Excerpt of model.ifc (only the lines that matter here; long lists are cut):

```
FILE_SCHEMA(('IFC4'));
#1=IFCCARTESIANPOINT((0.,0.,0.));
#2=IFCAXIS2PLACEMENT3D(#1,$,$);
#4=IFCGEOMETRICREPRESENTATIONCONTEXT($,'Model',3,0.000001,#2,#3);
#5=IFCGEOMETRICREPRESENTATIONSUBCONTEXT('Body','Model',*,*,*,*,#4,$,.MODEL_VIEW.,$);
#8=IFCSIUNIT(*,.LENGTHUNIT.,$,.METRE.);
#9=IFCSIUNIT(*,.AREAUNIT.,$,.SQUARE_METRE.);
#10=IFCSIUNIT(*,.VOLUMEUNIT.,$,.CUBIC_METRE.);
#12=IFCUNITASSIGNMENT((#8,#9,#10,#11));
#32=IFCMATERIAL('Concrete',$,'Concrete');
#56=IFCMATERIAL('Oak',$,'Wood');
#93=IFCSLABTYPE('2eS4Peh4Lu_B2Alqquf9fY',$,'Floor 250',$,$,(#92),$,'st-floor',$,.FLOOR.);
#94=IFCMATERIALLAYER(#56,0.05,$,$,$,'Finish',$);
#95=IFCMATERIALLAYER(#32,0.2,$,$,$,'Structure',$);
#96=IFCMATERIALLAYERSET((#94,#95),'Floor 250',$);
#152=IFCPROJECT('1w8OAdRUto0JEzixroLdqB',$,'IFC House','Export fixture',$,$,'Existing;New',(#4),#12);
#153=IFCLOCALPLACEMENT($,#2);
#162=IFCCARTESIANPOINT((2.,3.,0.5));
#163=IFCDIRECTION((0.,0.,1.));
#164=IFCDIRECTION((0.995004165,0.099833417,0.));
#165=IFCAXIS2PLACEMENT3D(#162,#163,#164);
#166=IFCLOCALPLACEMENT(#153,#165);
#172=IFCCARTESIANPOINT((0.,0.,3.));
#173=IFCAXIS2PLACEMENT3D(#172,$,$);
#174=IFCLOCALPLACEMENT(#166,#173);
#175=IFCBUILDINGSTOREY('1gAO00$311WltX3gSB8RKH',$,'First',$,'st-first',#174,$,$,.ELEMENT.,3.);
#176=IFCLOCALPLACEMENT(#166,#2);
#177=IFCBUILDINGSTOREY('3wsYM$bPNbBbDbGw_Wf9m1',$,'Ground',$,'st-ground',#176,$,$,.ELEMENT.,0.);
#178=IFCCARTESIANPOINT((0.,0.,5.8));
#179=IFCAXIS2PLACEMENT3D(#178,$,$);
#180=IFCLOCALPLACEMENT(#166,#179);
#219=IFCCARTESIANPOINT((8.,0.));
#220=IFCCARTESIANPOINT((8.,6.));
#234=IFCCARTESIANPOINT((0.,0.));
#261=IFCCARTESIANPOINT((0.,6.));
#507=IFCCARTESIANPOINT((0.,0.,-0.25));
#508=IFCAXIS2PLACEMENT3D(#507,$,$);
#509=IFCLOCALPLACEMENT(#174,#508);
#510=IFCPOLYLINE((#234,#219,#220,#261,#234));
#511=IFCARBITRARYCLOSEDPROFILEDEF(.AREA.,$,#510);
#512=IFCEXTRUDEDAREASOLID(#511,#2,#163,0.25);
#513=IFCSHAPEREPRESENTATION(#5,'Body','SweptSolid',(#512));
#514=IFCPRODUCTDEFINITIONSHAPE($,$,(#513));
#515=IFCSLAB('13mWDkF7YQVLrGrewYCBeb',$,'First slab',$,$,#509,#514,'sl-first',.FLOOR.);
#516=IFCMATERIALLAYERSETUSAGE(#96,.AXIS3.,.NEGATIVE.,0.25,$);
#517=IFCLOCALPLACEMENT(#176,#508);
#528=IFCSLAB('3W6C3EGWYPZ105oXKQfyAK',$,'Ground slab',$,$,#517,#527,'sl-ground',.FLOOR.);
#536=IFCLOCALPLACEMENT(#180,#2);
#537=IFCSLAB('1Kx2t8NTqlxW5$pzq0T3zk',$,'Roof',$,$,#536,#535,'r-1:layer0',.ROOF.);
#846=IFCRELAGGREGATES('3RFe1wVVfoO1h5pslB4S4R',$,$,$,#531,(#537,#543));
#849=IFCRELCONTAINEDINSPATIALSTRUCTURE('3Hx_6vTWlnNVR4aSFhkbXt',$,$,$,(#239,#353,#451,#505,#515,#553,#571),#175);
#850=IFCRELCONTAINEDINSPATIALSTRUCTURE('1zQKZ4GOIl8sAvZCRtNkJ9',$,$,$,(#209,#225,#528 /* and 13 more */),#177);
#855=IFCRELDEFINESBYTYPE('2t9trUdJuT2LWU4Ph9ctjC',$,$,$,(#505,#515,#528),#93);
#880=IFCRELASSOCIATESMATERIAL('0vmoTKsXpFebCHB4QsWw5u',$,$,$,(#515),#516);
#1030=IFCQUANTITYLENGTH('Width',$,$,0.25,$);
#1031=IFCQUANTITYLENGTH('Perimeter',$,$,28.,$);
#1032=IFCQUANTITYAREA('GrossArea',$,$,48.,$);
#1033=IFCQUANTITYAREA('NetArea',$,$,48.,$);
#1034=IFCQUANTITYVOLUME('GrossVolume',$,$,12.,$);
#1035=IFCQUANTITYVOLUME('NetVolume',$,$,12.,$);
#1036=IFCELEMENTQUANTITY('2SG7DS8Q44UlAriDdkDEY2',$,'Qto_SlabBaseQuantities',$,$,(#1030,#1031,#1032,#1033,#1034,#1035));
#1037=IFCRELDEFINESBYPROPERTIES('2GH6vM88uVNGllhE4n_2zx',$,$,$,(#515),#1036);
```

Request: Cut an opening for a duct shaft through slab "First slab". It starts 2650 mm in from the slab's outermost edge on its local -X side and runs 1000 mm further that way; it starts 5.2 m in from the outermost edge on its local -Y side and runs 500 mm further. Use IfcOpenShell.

```python
import numpy as np
import ifcopenshell
import ifcopenshell.api.feature
import ifcopenshell.api.geometry
import ifcopenshell.api.pset
import ifcopenshell.api.root
import ifcopenshell.geom
import ifcopenshell.util.element
import ifcopenshell.util.placement
import ifcopenshell.util.representation
import ifcopenshell.util.shape
import ifcopenshell.util.unit

model = ifcopenshell.open("model.ifc")
unit_scale = ifcopenshell.util.unit.calculate_unit_scale(model)
area_scale = ifcopenshell.util.unit.calculate_unit_scale(model, "AREAUNIT")
volume_scale = ifcopenshell.util.unit.calculate_unit_scale(model, "VOLUMEUNIT")
settings = ifcopenshell.geom.settings()


def volume(element):
    """Net volume in cubic metres, openings subtracted."""
    shape = ifcopenshell.geom.create_shape(settings, element)
    return ifcopenshell.util.shape.get_volume(shape.geometry)


slab = model.by_guid("13mWDkF7YQVLrGrewYCBeb")
before = volume(slab)

# Extent in the slab's own axes, in metres. The edges named are its -X and -Y sides.
slab_shape = ifcopenshell.geom.create_shape(settings, slab)
vertices = ifcopenshell.util.shape.get_vertices(slab_shape.geometry)
x_min, y_min, bottom = vertices.min(axis=0)
top = vertices[:, 2].max()

opening = ifcopenshell.api.root.create_entity(model, ifc_class="IfcOpeningElement", name="Duct shaft opening", predefined_type="OPENING")
context = ifcopenshell.util.representation.get_context(model, "Model", "Body", "MODEL_VIEW")
width, depth = 1, 0.5
outline = [(0.0, 0.0), (width, 0.0), (width, depth), (0.0, depth), (0.0, 0.0)]
# Overshoot both faces by 50 mm so the cut is clean.
shape = ifcopenshell.api.geometry.add_slab_representation(
    model, context=context, depth=top - bottom + 0.1, polyline=outline
)
ifcopenshell.api.geometry.assign_representation(model, product=opening, representation=shape)

matrix = ifcopenshell.util.placement.get_local_placement(slab.ObjectPlacement)
matrix[:, 3] = matrix @ np.append(np.array([x_min + 2.65, y_min + 5.2, bottom - 0.05]) / unit_scale, 1.0)
ifcopenshell.api.geometry.edit_object_placement(model, product=opening, matrix=matrix, is_si=False)
ifcopenshell.api.feature.add_feature(model, feature=opening, element=slab)

after = volume(slab)

# Update the slab's stored quantities.
qto = model.by_id(ifcopenshell.util.element.get_pset(slab, "Qto_SlabBaseQuantities", should_inherit=False)["id"])
ifcopenshell.api.pset.edit_qto(model, qto=qto, properties={
    "NetArea": after / (top - bottom) / area_scale,
    "NetVolume": after / volume_scale,
})

print(f"slab volume {before:.3f} -> {after:.3f} m3")

model.write("model_updated.ifc")
```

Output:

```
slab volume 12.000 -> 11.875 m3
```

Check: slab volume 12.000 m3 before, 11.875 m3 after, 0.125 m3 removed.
